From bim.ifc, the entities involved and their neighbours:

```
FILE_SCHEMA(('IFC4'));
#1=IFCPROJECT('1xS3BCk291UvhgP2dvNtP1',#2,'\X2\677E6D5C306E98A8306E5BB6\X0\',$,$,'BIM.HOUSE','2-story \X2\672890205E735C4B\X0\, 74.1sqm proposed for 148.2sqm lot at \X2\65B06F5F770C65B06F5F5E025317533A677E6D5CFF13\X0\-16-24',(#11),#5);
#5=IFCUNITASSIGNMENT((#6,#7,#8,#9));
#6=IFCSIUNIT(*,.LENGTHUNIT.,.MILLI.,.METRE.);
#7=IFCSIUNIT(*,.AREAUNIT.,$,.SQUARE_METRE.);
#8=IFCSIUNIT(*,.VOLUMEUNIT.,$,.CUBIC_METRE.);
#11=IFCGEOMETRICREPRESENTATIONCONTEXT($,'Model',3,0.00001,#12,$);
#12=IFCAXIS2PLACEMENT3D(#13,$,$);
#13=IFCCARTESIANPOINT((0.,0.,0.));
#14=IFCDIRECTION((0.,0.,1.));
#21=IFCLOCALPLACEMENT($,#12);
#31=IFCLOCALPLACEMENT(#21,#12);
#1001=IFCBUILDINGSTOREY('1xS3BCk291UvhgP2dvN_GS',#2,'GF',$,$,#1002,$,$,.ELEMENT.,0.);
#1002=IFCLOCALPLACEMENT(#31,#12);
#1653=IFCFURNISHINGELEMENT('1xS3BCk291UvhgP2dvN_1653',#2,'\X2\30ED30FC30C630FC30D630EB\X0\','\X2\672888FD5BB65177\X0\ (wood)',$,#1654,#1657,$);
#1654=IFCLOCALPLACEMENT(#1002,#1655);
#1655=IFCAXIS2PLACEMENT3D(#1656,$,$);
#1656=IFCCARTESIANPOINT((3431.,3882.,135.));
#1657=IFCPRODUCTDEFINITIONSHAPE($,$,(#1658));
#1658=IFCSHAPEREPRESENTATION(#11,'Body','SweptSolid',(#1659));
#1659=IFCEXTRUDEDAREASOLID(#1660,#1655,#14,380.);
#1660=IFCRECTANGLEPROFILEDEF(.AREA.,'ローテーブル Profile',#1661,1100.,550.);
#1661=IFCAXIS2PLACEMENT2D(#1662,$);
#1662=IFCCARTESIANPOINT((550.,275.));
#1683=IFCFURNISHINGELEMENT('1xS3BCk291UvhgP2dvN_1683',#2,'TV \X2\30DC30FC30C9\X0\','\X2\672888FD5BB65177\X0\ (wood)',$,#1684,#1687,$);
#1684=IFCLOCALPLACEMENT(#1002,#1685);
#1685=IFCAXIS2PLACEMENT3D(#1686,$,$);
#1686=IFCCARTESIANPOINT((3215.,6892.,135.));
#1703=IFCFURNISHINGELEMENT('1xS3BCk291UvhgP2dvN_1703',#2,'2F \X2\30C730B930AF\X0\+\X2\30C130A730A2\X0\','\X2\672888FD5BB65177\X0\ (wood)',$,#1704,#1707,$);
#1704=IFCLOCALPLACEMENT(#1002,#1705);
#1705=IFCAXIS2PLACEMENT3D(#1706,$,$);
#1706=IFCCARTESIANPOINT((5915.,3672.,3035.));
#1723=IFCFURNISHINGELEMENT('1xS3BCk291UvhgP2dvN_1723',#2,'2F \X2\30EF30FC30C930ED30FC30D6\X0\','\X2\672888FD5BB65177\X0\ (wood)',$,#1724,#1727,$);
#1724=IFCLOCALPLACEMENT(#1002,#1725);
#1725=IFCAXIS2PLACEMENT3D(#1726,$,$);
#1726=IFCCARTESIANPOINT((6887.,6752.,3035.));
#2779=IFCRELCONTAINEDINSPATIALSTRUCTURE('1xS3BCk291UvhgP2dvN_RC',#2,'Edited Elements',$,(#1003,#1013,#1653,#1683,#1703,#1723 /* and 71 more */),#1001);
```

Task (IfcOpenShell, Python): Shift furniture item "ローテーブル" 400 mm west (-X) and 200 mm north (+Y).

```python
import ifcopenshell
import ifcopenshell.api.geometry
import ifcopenshell.util.placement

model = ifcopenshell.open("bim.ifc")

item = model.by_guid("1xS3BCk291UvhgP2dvN_1653")
matrix = ifcopenshell.util.placement.get_local_placement(item.ObjectPlacement)
matrix[0, 3] -= 400.0
matrix[1, 3] += 200.0
ifcopenshell.api.geometry.edit_object_placement(model, product=item, matrix=matrix, is_si=False)

print(ifcopenshell.util.placement.get_local_placement(item.ObjectPlacement).round(3) + 0.0)

model.write("bim-out.ifc")
```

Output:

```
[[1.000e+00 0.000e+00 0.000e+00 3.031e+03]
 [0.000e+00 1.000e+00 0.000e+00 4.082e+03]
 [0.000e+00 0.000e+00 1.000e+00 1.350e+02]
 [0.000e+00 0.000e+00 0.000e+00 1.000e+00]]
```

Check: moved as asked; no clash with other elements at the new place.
